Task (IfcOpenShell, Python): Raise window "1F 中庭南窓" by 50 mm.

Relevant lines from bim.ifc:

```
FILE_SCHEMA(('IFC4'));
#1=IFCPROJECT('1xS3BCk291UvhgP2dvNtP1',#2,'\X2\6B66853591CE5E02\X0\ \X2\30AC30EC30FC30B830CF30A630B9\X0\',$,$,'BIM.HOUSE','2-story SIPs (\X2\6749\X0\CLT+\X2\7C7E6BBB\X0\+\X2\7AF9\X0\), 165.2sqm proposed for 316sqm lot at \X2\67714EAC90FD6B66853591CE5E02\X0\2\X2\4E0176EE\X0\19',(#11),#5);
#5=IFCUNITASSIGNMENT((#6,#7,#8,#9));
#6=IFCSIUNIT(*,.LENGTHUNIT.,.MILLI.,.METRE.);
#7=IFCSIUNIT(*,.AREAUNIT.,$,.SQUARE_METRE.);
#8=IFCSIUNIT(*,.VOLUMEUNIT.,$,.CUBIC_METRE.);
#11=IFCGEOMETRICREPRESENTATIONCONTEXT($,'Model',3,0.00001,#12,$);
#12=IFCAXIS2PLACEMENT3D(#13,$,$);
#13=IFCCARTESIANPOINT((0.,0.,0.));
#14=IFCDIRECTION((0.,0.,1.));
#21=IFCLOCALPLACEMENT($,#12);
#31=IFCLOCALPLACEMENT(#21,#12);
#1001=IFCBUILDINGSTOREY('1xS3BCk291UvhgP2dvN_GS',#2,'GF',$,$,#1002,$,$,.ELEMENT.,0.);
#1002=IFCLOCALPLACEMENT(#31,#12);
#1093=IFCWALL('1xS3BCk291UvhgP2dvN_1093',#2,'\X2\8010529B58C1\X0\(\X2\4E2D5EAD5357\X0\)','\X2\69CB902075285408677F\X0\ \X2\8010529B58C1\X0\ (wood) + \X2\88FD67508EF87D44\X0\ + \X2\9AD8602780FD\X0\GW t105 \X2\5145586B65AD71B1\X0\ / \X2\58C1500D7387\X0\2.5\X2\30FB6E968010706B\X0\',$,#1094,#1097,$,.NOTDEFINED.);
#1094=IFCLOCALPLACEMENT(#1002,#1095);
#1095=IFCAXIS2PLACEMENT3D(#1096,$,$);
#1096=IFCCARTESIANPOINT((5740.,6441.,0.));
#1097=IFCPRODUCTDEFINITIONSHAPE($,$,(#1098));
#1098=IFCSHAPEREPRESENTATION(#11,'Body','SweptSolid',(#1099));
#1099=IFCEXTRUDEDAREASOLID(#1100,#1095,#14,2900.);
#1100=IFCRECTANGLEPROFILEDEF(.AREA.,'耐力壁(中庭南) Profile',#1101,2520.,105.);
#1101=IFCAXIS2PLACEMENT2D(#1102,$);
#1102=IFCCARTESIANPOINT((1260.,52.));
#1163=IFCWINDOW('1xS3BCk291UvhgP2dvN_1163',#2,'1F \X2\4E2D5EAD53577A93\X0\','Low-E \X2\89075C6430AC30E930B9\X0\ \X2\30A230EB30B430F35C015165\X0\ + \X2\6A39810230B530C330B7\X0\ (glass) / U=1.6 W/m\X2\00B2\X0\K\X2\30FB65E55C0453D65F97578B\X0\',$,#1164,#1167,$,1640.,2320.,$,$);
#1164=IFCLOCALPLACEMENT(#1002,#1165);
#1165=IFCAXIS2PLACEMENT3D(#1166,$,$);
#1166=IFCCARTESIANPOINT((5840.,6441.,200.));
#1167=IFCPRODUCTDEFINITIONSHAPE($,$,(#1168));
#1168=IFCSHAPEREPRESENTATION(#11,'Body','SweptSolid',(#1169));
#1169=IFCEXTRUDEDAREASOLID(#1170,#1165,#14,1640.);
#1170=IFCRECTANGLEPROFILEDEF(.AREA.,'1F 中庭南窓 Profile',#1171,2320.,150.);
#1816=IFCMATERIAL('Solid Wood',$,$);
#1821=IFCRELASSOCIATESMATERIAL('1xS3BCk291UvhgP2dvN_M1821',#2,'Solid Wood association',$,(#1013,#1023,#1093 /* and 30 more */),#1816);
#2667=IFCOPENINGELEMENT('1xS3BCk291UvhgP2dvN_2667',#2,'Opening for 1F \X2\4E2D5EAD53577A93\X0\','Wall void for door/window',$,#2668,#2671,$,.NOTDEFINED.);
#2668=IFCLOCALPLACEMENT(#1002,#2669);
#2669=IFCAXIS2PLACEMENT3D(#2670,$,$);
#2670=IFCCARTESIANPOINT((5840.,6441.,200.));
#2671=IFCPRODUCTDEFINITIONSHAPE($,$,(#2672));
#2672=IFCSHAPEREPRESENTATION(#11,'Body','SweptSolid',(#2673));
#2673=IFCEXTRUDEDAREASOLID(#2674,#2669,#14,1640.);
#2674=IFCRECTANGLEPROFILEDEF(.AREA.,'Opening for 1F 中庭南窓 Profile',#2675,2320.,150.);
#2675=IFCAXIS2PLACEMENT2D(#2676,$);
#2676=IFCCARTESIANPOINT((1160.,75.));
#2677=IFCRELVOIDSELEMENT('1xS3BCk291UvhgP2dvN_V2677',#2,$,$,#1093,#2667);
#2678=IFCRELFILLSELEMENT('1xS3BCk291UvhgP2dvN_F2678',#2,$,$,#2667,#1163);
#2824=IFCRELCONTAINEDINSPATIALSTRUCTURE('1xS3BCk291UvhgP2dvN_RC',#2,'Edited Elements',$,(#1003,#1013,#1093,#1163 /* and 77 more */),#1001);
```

```python
import numpy as np
import ifcopenshell
import ifcopenshell.api.geometry
import ifcopenshell.util.placement
import ifcopenshell.util.unit

model = ifcopenshell.open("bim.ifc")
unit_scale = ifcopenshell.util.unit.calculate_unit_scale(model)

window = model.by_id(1163)
opening = window.FillsVoids[0].RelatingOpeningElement
dz = 0.05 / unit_scale

shift = np.array([0.0, 0.0, dz])
# The window is not placed relative to its opening, so move both.
for product in (opening, window):
    matrix = ifcopenshell.util.placement.get_local_placement(product.ObjectPlacement)
    matrix[:3, 3] += shift
    ifcopenshell.api.geometry.edit_object_placement(model, product=product, matrix=matrix, is_si=False)

print(f"moved by {dz * unit_scale:+.3f} m")

model.write("bim-out.ifc")
```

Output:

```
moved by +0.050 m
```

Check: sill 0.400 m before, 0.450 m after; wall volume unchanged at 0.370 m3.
